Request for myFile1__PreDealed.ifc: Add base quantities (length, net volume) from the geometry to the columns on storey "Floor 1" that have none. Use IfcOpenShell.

First a look at what the model holds.

```python
import ifcopenshell
import ifcopenshell.util.element
import ifcopenshell.util.unit

model = ifcopenshell.open("myFile1__PreDealed.ifc")
print(model.schema)
for unit_type in ("LENGTHUNIT", "AREAUNIT", "VOLUMEUNIT"):
    print(unit_type, ifcopenshell.util.unit.calculate_unit_scale(model, unit_type))
storey = next(s for s in model.by_type("IfcBuildingStorey") if s.Name == "Floor 1")
columns = [e for e in ifcopenshell.util.element.get_decomposition(storey) if e.is_a("IfcColumn")]
for e in sorted(columns, key=lambda e: e.id()):
    print(e.id(), e.is_a(), e.Name, list(ifcopenshell.util.element.get_psets(e, qtos_only=True)), sep=" | ")
```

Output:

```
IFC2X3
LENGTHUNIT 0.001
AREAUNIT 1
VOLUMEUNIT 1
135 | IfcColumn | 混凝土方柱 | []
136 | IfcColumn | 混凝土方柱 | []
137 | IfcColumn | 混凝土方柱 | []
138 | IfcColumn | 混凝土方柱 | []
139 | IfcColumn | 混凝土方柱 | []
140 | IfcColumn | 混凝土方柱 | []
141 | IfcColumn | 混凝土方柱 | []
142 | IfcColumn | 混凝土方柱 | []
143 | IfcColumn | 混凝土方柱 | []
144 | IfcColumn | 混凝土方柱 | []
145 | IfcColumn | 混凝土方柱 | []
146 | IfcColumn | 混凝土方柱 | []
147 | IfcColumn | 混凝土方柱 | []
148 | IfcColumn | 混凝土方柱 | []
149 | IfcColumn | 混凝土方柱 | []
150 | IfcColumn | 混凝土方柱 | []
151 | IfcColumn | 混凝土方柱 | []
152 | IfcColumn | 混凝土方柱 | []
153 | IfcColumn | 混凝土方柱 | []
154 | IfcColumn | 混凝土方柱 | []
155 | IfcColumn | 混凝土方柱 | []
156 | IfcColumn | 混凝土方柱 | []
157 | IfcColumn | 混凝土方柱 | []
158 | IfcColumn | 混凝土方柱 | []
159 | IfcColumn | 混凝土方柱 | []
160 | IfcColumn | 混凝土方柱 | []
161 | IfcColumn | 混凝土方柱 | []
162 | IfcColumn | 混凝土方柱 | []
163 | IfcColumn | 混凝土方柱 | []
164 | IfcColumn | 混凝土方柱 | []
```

```python
import ifcopenshell
import ifcopenshell.api.pset
import ifcopenshell.geom
import ifcopenshell.util.element
import ifcopenshell.util.shape
import ifcopenshell.util.unit

model = ifcopenshell.open("myFile1__PreDealed.ifc")
unit_scale = ifcopenshell.util.unit.calculate_unit_scale(model)
volume_scale = ifcopenshell.util.unit.calculate_unit_scale(model, "VOLUMEUNIT")
settings = ifcopenshell.geom.settings()

storey = next(s for s in model.by_type("IfcBuildingStorey") if s.Name == "Floor 1")
columns = [e for e in ifcopenshell.util.element.get_decomposition(storey) if e.is_a("IfcColumn")]

for e in sorted(columns, key=lambda e: e.id()):
    if ifcopenshell.util.element.get_psets(e, qtos_only=True, should_inherit=False):
        continue
    # Geometry comes back in metres, in the element's own axes.
    shape = ifcopenshell.geom.create_shape(settings, e)
    values = {
        "Length": ifcopenshell.util.shape.get_z(shape.geometry) / unit_scale,
        "NetVolume": ifcopenshell.util.shape.get_volume(shape.geometry) / volume_scale,
    }
    qto = ifcopenshell.api.pset.add_qto(model, product=e, name="BaseQuantities")
    ifcopenshell.api.pset.edit_qto(model, qto=qto, properties=values)
    print(e.id(), {k: round(v, 3) for k, v in values.items()})

model.write("myFile1__PreDealed-out.ifc")
```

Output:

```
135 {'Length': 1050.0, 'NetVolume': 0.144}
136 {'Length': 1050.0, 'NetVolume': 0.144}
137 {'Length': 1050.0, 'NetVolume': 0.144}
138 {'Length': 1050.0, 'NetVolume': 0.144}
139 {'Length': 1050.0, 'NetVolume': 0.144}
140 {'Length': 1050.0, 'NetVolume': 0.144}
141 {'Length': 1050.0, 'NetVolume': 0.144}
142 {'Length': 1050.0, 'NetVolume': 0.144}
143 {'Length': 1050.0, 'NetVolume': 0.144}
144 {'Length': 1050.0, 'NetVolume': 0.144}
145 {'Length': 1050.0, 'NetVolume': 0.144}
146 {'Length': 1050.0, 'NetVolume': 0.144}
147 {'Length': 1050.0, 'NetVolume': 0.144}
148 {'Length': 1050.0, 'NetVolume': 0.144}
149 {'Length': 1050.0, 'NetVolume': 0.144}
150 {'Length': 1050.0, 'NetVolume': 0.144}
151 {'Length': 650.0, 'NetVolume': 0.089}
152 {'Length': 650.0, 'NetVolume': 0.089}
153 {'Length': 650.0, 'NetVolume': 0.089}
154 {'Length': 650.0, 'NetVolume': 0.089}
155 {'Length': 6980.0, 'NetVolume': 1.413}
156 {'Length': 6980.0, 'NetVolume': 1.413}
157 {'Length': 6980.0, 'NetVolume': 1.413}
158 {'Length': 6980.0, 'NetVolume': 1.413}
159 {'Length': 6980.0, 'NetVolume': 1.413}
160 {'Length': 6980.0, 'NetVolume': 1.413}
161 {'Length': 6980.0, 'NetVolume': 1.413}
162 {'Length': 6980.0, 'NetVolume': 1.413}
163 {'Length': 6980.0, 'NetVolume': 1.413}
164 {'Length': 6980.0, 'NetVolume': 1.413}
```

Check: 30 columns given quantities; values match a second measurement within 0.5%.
